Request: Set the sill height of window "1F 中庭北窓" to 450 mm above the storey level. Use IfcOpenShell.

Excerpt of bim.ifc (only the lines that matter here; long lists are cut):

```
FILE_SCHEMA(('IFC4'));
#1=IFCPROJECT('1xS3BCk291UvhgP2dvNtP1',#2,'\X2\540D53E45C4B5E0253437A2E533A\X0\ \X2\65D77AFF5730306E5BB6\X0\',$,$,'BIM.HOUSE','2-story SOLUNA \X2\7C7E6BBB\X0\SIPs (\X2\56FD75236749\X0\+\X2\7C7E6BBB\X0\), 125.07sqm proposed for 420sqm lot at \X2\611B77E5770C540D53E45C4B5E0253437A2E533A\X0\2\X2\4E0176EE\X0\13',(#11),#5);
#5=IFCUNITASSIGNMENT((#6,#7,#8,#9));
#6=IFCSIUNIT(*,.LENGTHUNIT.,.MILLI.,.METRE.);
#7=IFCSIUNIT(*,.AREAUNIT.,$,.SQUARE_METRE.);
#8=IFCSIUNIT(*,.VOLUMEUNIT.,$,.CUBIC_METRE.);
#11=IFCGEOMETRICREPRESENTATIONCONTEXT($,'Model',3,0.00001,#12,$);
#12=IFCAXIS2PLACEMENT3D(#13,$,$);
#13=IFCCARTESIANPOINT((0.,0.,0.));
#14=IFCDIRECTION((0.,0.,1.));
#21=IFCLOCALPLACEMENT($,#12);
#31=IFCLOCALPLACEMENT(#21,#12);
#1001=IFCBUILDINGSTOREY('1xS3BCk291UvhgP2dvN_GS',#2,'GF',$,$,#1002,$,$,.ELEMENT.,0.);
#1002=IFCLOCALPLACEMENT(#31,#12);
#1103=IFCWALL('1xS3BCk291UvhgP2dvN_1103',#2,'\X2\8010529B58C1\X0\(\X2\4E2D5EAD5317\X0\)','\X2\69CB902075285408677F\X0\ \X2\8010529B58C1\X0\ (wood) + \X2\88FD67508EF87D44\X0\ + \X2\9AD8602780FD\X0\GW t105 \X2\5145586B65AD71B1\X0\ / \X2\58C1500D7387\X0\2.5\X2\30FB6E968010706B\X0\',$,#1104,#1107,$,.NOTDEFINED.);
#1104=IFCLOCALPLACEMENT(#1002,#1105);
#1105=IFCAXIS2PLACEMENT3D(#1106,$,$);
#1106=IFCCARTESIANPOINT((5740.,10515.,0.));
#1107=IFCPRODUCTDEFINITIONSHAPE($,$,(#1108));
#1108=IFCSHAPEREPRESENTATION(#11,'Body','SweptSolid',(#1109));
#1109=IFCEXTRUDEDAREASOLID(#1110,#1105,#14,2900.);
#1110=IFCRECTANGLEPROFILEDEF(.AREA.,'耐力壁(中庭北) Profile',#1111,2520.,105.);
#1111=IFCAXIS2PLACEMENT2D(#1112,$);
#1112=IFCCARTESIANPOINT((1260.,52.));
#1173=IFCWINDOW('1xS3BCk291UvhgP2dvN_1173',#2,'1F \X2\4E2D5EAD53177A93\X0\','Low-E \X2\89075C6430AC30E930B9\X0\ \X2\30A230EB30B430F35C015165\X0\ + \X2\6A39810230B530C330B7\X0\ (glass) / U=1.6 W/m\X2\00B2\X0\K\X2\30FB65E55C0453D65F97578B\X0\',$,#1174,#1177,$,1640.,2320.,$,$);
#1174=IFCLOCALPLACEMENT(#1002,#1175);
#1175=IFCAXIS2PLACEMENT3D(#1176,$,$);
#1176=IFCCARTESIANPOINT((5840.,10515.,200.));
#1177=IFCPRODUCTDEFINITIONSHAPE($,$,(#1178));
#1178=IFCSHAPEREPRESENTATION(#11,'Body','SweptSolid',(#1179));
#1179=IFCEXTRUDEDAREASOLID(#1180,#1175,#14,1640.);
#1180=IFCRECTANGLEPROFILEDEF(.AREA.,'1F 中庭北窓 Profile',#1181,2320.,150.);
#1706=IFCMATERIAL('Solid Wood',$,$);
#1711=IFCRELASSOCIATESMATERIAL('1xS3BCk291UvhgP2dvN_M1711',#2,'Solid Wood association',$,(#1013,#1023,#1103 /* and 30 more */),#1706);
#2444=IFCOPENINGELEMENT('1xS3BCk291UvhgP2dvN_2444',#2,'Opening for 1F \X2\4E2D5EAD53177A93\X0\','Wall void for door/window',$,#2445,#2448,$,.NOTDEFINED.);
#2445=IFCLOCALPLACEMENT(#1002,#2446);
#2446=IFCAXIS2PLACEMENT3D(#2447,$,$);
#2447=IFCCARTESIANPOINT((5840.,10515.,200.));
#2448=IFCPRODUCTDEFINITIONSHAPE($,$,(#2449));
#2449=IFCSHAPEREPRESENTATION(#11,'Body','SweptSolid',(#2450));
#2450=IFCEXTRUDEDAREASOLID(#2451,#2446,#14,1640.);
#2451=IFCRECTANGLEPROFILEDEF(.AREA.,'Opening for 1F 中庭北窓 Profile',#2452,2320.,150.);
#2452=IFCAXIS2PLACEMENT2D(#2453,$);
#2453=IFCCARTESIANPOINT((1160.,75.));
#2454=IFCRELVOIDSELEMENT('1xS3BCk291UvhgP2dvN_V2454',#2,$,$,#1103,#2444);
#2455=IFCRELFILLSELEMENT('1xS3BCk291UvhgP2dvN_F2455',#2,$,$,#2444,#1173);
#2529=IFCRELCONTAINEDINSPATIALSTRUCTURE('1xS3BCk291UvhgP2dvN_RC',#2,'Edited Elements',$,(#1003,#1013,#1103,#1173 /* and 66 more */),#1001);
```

```python
import numpy as np
import ifcopenshell
import ifcopenshell.api.geometry
import ifcopenshell.geom
import ifcopenshell.util.element
import ifcopenshell.util.placement
import ifcopenshell.util.shape
import ifcopenshell.util.unit

model = ifcopenshell.open("bim.ifc")
unit_scale = ifcopenshell.util.unit.calculate_unit_scale(model)

window = model.by_guid("1xS3BCk291UvhgP2dvN_1173")
opening = window.FillsVoids[0].RelatingOpeningElement
storey = ifcopenshell.util.element.get_container(window, ifc_class="IfcBuildingStorey")
level = ifcopenshell.util.placement.get_local_placement(storey.ObjectPlacement)[2, 3]

# The opening's origin need not be at the sill, so measure its lowest point.
shape = ifcopenshell.geom.create_shape(ifcopenshell.geom.settings(), opening)
bottom = ifcopenshell.util.shape.get_shape_bottom_elevation(shape, shape.geometry) / unit_scale
dz = level + 450.0 - bottom

shift = np.array([0.0, 0.0, dz])
# The window is not placed relative to its opening, so move both.
for product in (opening, window):
    matrix = ifcopenshell.util.placement.get_local_placement(product.ObjectPlacement)
    matrix[:3, 3] += shift
    ifcopenshell.api.geometry.edit_object_placement(model, product=product, matrix=matrix, is_si=False)

print(f"moved by {dz * unit_scale:+.3f} m")

model.write("bim_rev.ifc")
```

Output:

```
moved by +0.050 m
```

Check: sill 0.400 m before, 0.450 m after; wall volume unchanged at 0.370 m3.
